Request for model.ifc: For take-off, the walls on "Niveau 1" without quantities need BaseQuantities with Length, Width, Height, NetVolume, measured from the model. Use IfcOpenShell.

First a look at what the model holds.

```python
import ifcopenshell
import ifcopenshell.util.element
import ifcopenshell.util.unit

model = ifcopenshell.open("model.ifc")
print(model.schema)
for unit_type in ("LENGTHUNIT", "AREAUNIT", "VOLUMEUNIT"):
    print(unit_type, ifcopenshell.util.unit.calculate_unit_scale(model, unit_type))
storey = next(s for s in model.by_type("IfcBuildingStorey") if s.Name == "Niveau 1")
walls = [e for e in ifcopenshell.util.element.get_decomposition(storey) if e.is_a("IfcWall")]
for e in sorted(walls, key=lambda e: e.id()):
    print(e.id(), e.is_a(), e.Name, list(ifcopenshell.util.element.get_psets(e, qtos_only=True)), sep=" | ")
```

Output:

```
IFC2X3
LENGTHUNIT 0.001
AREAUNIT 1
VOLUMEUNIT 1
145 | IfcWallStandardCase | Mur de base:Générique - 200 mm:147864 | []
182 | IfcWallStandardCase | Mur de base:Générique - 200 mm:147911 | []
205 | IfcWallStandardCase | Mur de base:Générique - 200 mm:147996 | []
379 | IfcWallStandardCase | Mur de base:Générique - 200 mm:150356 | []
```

```python
import ifcopenshell
import ifcopenshell.api.pset
import ifcopenshell.geom
import ifcopenshell.util.element
import ifcopenshell.util.shape
import ifcopenshell.util.unit

model = ifcopenshell.open("model.ifc")
unit_scale = ifcopenshell.util.unit.calculate_unit_scale(model)
volume_scale = ifcopenshell.util.unit.calculate_unit_scale(model, "VOLUMEUNIT")
settings = ifcopenshell.geom.settings()

storey = next(s for s in model.by_type("IfcBuildingStorey") if s.Name == "Niveau 1")
walls = [e for e in ifcopenshell.util.element.get_decomposition(storey) if e.is_a("IfcWall")]

for e in sorted(walls, key=lambda e: e.id()):
    if ifcopenshell.util.element.get_psets(e, qtos_only=True, should_inherit=False):
        continue
    # Geometry comes back in metres, in the element's own axes.
    shape = ifcopenshell.geom.create_shape(settings, e)
    values = {
        "Length": ifcopenshell.util.shape.get_x(shape.geometry) / unit_scale,
        "Width": ifcopenshell.util.shape.get_y(shape.geometry) / unit_scale,
        "Height": ifcopenshell.util.shape.get_z(shape.geometry) / unit_scale,
        "NetVolume": ifcopenshell.util.shape.get_volume(shape.geometry) / volume_scale,
    }
    qto = ifcopenshell.api.pset.add_qto(model, product=e, name="BaseQuantities")
    ifcopenshell.api.pset.edit_qto(model, qto=qto, properties=values)
    print(e.id(), {k: round(v, 3) for k, v in values.items()})

model.write("model_v2.ifc")
```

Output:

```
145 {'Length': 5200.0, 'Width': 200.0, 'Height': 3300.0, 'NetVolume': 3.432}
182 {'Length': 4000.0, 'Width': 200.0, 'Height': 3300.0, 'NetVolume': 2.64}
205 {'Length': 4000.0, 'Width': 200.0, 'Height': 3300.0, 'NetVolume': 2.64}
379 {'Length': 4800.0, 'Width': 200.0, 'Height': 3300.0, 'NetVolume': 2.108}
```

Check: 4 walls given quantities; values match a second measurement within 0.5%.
